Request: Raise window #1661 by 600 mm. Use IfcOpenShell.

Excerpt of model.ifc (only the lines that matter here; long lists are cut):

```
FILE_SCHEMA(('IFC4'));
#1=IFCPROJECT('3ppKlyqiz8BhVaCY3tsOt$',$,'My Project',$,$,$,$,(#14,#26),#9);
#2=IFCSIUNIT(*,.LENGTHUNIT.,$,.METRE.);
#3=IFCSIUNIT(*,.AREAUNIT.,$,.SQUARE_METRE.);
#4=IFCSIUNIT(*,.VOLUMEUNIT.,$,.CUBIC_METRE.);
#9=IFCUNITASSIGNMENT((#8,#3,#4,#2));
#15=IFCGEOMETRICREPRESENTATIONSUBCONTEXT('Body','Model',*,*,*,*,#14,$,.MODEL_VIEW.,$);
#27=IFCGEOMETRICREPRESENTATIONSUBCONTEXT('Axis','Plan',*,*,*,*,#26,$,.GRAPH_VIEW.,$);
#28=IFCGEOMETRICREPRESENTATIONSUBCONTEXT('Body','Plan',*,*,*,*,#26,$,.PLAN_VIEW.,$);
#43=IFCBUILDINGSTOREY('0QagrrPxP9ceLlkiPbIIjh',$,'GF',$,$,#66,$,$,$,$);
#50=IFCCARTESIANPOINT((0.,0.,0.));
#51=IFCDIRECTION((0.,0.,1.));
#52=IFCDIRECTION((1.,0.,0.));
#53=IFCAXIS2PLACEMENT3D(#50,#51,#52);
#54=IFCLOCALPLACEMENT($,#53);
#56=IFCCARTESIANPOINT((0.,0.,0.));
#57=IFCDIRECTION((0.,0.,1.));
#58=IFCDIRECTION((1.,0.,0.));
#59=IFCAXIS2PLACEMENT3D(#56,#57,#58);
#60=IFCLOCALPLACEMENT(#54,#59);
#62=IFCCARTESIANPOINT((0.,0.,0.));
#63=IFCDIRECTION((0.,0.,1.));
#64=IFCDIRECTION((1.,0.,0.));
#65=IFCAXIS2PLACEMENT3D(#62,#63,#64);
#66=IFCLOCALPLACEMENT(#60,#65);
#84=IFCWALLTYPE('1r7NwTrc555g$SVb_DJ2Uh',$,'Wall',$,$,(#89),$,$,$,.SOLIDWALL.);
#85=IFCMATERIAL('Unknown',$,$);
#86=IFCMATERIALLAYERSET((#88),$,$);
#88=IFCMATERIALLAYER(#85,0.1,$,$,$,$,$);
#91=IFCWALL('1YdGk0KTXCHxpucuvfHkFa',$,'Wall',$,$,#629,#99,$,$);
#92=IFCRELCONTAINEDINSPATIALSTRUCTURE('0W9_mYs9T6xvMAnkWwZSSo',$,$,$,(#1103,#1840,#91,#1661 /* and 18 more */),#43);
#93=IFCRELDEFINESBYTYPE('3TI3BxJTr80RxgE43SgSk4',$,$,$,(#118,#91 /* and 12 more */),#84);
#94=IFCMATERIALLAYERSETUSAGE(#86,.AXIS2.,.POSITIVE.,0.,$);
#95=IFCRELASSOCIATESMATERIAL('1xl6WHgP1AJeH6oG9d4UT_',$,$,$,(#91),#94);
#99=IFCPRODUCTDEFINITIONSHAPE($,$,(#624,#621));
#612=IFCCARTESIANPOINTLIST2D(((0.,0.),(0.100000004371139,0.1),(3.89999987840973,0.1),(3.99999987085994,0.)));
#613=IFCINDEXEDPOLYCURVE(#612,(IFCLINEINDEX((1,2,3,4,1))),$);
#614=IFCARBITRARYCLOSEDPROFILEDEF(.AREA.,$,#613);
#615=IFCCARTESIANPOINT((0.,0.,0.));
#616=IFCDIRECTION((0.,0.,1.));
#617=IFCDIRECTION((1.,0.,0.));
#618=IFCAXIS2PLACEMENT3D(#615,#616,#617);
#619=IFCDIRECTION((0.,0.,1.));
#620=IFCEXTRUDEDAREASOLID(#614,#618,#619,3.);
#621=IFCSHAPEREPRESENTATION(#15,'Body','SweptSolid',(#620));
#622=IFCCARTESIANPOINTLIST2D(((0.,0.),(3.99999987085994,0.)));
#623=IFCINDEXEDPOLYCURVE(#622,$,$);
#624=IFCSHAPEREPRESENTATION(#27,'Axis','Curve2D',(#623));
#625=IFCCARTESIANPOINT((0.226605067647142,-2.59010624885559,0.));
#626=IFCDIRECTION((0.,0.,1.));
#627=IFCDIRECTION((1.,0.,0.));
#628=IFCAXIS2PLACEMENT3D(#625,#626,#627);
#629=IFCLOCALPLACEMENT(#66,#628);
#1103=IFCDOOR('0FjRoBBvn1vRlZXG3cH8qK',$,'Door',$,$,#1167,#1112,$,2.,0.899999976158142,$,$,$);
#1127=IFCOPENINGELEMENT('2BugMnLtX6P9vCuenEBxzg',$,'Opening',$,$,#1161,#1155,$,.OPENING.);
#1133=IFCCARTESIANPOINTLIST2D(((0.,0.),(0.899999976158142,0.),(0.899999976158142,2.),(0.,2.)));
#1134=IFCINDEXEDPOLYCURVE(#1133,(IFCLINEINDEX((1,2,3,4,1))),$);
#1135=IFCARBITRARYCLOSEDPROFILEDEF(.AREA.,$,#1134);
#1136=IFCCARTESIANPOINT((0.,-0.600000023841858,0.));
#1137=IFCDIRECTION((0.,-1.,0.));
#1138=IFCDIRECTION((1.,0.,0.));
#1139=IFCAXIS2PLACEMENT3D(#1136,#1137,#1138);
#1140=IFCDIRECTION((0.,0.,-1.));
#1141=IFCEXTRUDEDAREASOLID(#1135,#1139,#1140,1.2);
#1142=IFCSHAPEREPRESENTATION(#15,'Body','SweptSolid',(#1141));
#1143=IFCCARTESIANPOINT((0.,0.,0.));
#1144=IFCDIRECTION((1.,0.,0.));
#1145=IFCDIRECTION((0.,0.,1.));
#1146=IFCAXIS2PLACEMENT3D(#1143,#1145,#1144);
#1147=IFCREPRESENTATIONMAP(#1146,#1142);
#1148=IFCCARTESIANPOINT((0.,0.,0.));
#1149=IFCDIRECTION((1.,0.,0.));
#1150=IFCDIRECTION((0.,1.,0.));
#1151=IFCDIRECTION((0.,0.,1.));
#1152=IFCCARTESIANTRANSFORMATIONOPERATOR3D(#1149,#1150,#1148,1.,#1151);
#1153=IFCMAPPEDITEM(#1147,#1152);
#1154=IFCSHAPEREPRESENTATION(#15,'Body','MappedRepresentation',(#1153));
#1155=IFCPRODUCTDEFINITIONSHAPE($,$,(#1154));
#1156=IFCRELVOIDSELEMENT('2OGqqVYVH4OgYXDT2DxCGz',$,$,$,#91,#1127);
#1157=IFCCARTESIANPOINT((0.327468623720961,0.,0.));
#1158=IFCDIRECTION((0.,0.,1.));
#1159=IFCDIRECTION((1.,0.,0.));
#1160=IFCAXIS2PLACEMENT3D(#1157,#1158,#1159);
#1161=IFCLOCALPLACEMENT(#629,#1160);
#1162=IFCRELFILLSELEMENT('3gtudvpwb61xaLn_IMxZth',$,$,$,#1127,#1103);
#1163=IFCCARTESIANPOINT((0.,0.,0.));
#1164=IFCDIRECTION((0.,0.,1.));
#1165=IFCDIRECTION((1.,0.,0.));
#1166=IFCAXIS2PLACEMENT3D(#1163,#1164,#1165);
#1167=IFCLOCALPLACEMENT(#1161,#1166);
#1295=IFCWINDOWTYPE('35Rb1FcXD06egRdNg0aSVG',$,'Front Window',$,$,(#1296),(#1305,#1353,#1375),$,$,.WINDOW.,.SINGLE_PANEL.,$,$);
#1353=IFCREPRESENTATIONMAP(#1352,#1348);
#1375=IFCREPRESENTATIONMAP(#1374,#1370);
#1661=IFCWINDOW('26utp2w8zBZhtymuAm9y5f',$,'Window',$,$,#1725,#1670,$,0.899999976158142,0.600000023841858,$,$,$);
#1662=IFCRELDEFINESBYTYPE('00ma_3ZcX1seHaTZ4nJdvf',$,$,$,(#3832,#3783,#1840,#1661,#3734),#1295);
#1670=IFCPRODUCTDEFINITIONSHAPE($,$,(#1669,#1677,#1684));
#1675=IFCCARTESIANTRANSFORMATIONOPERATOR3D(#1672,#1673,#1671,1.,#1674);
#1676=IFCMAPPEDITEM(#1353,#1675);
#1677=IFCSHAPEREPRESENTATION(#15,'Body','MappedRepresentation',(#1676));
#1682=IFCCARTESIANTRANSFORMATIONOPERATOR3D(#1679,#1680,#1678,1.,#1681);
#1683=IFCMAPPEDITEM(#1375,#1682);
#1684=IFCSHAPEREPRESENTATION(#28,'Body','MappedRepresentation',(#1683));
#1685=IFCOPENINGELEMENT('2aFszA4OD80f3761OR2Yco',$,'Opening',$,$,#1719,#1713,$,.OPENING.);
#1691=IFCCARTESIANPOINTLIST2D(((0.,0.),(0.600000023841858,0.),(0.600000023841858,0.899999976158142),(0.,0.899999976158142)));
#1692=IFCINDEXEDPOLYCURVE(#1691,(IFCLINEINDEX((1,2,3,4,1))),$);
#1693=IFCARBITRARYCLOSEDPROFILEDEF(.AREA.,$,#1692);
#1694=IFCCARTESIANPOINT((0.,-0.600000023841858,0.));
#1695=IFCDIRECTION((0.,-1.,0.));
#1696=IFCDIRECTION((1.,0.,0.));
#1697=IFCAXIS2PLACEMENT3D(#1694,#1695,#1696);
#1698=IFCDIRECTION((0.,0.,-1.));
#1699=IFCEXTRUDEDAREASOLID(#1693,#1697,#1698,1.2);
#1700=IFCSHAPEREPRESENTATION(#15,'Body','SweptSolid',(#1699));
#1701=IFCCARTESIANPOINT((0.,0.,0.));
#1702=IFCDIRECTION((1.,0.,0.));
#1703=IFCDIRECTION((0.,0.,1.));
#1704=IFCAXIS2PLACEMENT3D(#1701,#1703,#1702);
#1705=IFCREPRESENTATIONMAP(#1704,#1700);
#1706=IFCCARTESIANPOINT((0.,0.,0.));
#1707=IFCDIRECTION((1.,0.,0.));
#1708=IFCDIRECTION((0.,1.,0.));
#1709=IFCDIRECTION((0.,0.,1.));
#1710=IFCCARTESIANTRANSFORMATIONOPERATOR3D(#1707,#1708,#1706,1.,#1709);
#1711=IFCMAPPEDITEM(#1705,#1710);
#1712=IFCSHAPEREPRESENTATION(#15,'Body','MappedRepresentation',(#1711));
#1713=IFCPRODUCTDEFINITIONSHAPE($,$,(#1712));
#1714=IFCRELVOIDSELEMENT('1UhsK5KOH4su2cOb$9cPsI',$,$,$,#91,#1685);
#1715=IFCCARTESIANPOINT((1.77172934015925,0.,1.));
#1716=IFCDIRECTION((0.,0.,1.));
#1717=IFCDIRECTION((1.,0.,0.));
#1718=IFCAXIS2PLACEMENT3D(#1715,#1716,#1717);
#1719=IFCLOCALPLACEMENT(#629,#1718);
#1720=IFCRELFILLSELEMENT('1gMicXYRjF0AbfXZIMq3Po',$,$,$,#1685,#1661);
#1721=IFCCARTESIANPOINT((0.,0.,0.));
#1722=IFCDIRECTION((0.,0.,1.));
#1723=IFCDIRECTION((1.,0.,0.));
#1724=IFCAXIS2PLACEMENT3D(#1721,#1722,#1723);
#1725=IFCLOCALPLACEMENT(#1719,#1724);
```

```python
import numpy as np
import ifcopenshell
import ifcopenshell.api.geometry
import ifcopenshell.util.placement
import ifcopenshell.util.unit

model = ifcopenshell.open("model.ifc")
unit_scale = ifcopenshell.util.unit.calculate_unit_scale(model)

window = model.by_guid("26utp2w8zBZhtymuAm9y5f")
opening = window.FillsVoids[0].RelatingOpeningElement
dz = 0.6

shift = np.array([0.0, 0.0, dz])
# The window is placed relative to its opening, so it follows when the opening moves.
matrix = ifcopenshell.util.placement.get_local_placement(opening.ObjectPlacement)
matrix[:3, 3] += shift
ifcopenshell.api.geometry.edit_object_placement(
    model, product=opening, matrix=matrix, is_si=False, should_transform_children=True
)

print(f"moved by {dz * unit_scale:+.3f} m")

model.write("model-out.ifc")
```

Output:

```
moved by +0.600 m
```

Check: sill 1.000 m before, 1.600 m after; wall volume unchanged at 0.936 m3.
